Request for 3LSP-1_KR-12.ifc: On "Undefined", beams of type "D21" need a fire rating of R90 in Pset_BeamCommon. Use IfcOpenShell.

First a look at what the model holds.

```python
import ifcopenshell
import ifcopenshell.util.element

model = ifcopenshell.open("3LSP-1_KR-12.ifc")
print(model.schema)
storey = next(s for s in model.by_type("IfcBuildingStorey") if s.Name == "Undefined")
beams = [e for e in ifcopenshell.util.element.get_decomposition(storey) if e.is_a("IfcBeam")]
seen = {}
for e in beams:
    element_type = ifcopenshell.util.element.get_type(e)
    key = (element_type.Name if element_type != e and element_type else None, ifcopenshell.util.element.get_pset(e, "Pset_BeamCommon", "FireRating"))
    seen[key] = seen.get(key, 0) + 1
for (name, value), count in sorted(seen.items(), key=str):
    print(count, "x", name, "|", value)
```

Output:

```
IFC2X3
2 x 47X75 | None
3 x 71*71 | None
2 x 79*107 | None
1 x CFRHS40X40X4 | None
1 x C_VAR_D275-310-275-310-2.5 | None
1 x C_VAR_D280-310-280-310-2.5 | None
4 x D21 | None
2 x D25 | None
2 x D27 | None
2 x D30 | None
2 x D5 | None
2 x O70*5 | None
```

```python
import ifcopenshell
import ifcopenshell.api.pset
import ifcopenshell.util.element

model = ifcopenshell.open("3LSP-1_KR-12.ifc")

storey = next(s for s in model.by_type("IfcBuildingStorey") if s.Name == "Undefined")
beams = [e for e in ifcopenshell.util.element.get_decomposition(storey) if e.is_a("IfcBeam")]

count = 0
for e in beams:
    element_type = ifcopenshell.util.element.get_type(e)
    if element_type in (None, e) or element_type.Name != "D21":
        continue
    found = ifcopenshell.util.element.get_pset(e, "Pset_BeamCommon", should_inherit=False)
    if found:
        pset = model.by_id(found["id"])
        if len(ifcopenshell.util.element.get_elements_by_pset(pset)) > 1:
            pset = ifcopenshell.api.pset.unshare_pset(model, products=[e], pset=pset)[0]
    else:
        pset = ifcopenshell.api.pset.add_pset(model, product=e, name="Pset_BeamCommon")
    ifcopenshell.api.pset.edit_pset(model, pset=pset, properties={"FireRating": "R90"})
    count += 1

print(count, "beams updated")

model.write("3LSP-1_KR-12_updated.ifc")
```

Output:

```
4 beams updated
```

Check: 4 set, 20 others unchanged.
